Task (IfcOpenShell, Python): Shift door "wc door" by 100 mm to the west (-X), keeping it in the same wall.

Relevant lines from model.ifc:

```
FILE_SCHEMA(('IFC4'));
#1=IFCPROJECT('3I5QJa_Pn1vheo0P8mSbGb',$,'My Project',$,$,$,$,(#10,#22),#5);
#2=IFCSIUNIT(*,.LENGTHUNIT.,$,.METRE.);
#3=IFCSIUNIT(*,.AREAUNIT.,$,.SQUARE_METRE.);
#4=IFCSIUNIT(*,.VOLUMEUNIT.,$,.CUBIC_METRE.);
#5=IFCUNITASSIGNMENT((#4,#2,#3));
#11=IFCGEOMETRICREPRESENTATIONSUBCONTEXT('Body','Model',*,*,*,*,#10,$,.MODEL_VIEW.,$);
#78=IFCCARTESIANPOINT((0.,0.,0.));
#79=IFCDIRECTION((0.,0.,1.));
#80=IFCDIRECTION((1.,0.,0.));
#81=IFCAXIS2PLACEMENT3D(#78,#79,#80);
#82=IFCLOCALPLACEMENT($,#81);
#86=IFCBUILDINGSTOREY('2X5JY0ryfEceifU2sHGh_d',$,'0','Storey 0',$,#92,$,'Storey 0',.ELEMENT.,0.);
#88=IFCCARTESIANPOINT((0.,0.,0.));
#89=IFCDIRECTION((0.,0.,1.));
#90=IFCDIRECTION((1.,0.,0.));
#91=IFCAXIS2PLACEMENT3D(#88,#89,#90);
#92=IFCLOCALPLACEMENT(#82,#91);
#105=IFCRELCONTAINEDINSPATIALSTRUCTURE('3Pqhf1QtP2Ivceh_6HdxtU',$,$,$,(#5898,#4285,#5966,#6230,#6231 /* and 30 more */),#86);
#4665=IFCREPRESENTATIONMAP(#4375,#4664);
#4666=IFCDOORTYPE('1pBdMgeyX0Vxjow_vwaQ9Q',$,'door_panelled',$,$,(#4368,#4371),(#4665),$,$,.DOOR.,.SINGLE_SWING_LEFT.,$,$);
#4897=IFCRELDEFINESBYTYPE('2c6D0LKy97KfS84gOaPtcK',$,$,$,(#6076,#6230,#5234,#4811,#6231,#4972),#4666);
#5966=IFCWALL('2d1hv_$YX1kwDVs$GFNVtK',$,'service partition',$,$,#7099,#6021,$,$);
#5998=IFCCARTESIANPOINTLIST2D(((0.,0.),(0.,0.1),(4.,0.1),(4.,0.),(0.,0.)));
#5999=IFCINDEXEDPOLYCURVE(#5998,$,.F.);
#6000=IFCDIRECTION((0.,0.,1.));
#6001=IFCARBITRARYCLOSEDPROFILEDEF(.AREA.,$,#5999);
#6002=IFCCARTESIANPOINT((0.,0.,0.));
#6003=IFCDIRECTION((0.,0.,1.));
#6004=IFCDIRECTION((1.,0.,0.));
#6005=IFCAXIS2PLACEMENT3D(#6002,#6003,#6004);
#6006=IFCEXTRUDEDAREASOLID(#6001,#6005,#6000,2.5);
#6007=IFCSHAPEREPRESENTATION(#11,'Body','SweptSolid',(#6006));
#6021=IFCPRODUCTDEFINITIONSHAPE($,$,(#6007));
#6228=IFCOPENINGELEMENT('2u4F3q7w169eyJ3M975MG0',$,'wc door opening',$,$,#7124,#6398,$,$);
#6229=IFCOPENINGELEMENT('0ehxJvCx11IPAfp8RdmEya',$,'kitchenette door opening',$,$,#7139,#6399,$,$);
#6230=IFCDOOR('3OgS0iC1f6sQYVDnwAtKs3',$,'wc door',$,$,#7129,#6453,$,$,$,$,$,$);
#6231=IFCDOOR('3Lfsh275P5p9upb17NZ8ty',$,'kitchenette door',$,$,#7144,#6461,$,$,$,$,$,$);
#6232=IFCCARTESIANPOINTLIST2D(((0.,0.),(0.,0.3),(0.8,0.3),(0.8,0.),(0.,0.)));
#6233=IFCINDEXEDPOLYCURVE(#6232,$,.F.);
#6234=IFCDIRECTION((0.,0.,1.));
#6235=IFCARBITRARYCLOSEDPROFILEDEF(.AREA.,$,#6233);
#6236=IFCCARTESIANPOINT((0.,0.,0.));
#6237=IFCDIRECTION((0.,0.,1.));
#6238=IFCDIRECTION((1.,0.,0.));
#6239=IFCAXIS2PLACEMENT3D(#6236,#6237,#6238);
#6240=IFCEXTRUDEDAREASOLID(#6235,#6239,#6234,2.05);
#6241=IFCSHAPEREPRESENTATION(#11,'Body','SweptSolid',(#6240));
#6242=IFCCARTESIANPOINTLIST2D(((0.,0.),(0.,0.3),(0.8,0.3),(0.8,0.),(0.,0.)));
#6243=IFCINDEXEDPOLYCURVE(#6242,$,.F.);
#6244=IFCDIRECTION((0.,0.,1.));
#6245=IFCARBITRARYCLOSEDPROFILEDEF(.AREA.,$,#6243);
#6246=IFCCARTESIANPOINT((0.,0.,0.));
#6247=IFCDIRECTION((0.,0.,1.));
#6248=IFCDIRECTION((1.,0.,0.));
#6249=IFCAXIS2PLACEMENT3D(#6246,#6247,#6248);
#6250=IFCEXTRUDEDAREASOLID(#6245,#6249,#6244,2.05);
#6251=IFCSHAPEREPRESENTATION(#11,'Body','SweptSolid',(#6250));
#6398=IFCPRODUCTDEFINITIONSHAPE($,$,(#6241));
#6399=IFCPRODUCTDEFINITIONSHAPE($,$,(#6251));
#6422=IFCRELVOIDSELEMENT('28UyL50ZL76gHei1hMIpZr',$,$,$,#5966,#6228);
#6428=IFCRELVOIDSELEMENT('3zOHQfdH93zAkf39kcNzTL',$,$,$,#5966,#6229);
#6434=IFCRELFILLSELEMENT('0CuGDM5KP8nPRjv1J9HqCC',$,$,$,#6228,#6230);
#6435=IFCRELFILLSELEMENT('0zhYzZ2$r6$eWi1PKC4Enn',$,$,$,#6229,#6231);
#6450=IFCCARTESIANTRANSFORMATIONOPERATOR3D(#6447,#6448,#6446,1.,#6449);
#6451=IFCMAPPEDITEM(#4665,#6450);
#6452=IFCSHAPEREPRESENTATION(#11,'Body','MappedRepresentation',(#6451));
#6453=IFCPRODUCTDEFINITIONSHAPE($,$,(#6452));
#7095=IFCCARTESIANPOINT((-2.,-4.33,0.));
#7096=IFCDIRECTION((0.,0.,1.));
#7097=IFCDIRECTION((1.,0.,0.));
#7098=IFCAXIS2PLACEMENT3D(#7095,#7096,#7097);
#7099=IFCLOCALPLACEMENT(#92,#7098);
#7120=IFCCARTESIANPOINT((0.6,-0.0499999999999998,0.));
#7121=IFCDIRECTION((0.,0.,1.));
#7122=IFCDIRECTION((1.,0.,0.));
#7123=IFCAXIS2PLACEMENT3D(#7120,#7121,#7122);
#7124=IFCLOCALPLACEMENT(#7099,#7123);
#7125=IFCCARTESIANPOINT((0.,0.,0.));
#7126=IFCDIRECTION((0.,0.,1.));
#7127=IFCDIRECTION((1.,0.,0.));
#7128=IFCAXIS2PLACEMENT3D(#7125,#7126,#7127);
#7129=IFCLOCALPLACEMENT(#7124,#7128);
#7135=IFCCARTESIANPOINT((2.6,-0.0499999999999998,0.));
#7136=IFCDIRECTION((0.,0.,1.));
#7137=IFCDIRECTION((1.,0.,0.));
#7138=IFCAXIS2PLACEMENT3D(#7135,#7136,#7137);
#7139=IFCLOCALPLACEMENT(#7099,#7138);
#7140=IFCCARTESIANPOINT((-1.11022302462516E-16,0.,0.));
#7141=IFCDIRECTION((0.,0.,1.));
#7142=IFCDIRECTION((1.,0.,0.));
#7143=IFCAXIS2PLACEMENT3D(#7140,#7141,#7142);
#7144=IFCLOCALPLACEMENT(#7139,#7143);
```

```python
import ifcopenshell
import ifcopenshell.api.geometry
import ifcopenshell.util.placement
import ifcopenshell.util.unit

model = ifcopenshell.open("model.ifc")
unit_scale = ifcopenshell.util.unit.calculate_unit_scale(model)

door = model.by_guid("3OgS0iC1f6sQYVDnwAtKs3")
opening = door.FillsVoids[0].RelatingOpeningElement
wall = opening.VoidsElements[0].RelatingBuildingElement

wall_matrix = ifcopenshell.util.placement.get_local_placement(wall.ObjectPlacement)
shift = wall_matrix[:3, 0] * -0.1 / unit_scale
before = ifcopenshell.util.placement.get_local_placement(door.ObjectPlacement)[:3, 3].copy()

# The door is placed relative to its opening, so it follows when the opening moves.
matrix = ifcopenshell.util.placement.get_local_placement(opening.ObjectPlacement)
matrix[:3, 3] += shift
ifcopenshell.api.geometry.edit_object_placement(
    model, product=opening, matrix=matrix, is_si=False, should_transform_children=True
)

after = ifcopenshell.util.placement.get_local_placement(door.ObjectPlacement)[:3, 3]
print("door moved by", (after - before).round(3) + 0.0)

model.write("model_edited.ifc")
```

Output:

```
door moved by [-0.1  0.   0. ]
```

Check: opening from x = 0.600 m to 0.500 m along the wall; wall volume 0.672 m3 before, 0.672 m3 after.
